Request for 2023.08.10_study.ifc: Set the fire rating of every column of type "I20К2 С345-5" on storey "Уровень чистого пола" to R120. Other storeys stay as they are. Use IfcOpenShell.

First a look at what the model holds.

```python
import ifcopenshell
import ifcopenshell.util.element

model = ifcopenshell.open("2023.08.10_study.ifc")
print(model.schema)
storey = next(s for s in model.by_type("IfcBuildingStorey") if s.Name == "Уровень чистого пола")
columns = [e for e in ifcopenshell.util.element.get_decomposition(storey) if e.is_a("IfcColumn")]
seen = {}
for e in columns:
    element_type = ifcopenshell.util.element.get_type(e)
    key = (element_type.Name if element_type != e and element_type else None, ifcopenshell.util.element.get_pset(e, "Pset_ColumnCommon", "FireRating"))
    seen[key] = seen.get(key, 0) + 1
for (name, value), count in sorted(seen.items(), key=str):
    print(count, "x", name, "|", value)
```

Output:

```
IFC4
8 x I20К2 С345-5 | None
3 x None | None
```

```python
import ifcopenshell
import ifcopenshell.api.pset
import ifcopenshell.util.element

model = ifcopenshell.open("2023.08.10_study.ifc")

storey = next(s for s in model.by_type("IfcBuildingStorey") if s.Name == "Уровень чистого пола")
columns = [e for e in ifcopenshell.util.element.get_decomposition(storey) if e.is_a("IfcColumn")]

count = 0
for e in columns:
    element_type = ifcopenshell.util.element.get_type(e)
    if element_type in (None, e) or element_type.Name != "I20К2 С345-5":
        continue
    # add_pset returns the element's existing set when there is one.
    pset = ifcopenshell.api.pset.add_pset(model, product=e, name="Pset_ColumnCommon")
    ifcopenshell.api.pset.edit_pset(model, pset=pset, properties={"FireRating": "R120"})
    count += 1

print(count, "columns updated")

model.write("2023.08.10_study_v2.ifc")
```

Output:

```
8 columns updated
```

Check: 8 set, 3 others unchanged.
